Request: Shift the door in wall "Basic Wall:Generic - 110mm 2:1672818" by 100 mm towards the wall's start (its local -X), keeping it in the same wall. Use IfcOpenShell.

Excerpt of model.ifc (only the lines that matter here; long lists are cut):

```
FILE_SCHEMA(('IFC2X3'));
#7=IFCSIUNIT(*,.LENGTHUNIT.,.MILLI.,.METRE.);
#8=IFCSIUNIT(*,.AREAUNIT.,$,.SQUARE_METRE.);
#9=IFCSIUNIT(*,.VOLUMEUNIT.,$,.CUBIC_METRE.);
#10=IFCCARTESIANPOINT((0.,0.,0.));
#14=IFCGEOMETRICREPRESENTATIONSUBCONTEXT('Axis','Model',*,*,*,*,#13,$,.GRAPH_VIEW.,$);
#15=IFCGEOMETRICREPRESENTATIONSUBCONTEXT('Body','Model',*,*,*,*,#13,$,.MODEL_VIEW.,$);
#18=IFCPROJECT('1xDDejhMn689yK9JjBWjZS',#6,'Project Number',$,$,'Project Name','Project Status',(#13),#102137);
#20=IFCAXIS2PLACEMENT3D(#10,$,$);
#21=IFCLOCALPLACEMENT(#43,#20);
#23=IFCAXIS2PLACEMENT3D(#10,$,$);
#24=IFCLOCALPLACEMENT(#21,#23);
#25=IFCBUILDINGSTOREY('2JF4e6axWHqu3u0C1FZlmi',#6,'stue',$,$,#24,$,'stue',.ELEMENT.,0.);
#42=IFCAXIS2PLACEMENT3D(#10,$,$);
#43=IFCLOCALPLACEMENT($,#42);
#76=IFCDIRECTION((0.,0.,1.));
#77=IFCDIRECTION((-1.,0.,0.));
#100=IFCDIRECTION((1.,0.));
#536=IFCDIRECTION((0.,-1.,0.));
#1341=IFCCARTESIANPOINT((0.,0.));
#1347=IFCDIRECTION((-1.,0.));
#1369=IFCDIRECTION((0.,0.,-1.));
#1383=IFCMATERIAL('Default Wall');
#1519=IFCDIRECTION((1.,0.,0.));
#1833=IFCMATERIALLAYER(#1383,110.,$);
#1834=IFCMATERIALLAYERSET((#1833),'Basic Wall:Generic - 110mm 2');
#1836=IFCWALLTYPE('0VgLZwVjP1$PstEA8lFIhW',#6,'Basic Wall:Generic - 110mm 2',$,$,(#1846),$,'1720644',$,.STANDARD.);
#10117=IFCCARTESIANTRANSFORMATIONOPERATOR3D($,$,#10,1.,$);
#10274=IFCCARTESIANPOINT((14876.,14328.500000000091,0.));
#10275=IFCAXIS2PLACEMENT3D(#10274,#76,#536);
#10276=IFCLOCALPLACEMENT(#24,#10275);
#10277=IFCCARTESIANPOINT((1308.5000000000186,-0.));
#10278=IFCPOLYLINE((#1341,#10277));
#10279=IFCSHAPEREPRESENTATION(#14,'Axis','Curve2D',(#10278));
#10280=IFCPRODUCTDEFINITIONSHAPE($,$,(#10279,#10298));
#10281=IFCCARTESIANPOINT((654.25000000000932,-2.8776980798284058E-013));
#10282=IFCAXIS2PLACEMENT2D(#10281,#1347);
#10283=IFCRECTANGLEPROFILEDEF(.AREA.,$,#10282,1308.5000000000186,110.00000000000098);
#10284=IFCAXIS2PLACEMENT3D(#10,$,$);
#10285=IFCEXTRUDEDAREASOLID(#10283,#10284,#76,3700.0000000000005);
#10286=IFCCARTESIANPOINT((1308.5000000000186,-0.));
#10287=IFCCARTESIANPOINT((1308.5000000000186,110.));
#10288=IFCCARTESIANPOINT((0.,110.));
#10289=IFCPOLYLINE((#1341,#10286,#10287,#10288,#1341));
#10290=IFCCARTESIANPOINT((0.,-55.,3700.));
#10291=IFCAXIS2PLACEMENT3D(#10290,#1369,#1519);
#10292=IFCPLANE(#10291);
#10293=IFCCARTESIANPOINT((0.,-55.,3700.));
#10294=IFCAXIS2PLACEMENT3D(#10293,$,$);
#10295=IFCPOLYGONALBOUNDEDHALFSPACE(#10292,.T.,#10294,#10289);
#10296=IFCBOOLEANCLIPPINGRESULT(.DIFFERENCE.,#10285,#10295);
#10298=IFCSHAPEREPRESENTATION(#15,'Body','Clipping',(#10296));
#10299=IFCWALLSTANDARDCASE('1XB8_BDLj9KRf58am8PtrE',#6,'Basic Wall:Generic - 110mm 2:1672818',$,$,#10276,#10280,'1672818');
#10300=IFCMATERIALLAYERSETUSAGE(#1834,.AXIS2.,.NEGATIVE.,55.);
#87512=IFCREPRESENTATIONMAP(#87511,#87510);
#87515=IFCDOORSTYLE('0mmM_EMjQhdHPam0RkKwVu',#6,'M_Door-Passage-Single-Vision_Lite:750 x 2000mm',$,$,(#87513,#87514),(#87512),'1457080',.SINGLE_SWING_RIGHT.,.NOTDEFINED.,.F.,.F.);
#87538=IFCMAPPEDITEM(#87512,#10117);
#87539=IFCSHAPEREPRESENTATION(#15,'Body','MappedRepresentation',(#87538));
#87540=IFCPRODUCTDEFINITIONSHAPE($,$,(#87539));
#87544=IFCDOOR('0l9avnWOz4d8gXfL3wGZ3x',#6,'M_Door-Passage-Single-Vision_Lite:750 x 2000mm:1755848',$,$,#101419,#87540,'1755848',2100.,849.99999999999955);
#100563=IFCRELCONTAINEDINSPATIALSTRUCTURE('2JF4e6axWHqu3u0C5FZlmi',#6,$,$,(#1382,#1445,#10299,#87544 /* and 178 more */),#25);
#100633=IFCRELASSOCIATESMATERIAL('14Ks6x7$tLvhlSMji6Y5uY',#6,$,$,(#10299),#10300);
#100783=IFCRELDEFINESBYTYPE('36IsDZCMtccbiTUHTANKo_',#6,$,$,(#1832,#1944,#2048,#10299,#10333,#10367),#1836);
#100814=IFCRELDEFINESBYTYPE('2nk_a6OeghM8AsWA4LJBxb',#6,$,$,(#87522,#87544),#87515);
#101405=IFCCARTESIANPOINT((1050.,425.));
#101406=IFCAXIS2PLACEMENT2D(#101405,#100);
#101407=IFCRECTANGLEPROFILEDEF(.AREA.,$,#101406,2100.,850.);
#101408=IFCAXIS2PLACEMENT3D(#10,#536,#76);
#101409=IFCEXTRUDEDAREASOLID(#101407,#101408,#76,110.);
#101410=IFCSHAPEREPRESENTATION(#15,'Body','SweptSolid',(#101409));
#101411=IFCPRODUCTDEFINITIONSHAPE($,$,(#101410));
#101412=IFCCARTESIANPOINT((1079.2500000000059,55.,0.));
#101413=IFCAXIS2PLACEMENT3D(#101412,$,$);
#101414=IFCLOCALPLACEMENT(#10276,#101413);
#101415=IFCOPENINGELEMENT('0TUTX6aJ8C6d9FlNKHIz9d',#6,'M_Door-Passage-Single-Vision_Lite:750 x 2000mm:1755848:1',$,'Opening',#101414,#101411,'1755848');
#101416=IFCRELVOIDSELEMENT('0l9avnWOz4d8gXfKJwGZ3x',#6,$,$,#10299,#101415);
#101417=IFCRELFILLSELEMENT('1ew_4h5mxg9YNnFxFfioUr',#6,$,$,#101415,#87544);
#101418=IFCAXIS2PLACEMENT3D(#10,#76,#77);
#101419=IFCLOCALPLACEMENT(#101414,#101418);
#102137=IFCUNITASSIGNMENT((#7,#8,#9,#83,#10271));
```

```python
import ifcopenshell
import ifcopenshell.api.geometry
import ifcopenshell.util.placement

model = ifcopenshell.open("model.ifc")

door = model.by_guid("0l9avnWOz4d8gXfL3wGZ3x")
opening = door.FillsVoids[0].RelatingOpeningElement
wall = opening.VoidsElements[0].RelatingBuildingElement

wall_matrix = ifcopenshell.util.placement.get_local_placement(wall.ObjectPlacement)
shift = wall_matrix[:3, 0] * -100.0
before = ifcopenshell.util.placement.get_local_placement(door.ObjectPlacement)[:3, 3].copy()

# The door is placed relative to its opening, so it follows when the opening moves.
matrix = ifcopenshell.util.placement.get_local_placement(opening.ObjectPlacement)
matrix[:3, 3] += shift
ifcopenshell.api.geometry.edit_object_placement(
    model, product=opening, matrix=matrix, is_si=False, should_transform_children=True
)

after = ifcopenshell.util.placement.get_local_placement(door.ObjectPlacement)[:3, 3]
print("door moved by", (after - before).round(3) + 0.0)

model.write("model_edited.ifc")
```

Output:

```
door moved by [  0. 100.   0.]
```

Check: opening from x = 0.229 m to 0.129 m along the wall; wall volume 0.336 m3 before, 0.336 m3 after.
